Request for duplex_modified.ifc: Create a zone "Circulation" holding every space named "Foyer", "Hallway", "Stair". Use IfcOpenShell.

First a look at what the model holds.

```python
import ifcopenshell

model = ifcopenshell.open("duplex_modified.ifc")
print(model.schema)
seen = {}
for space in model.by_type("IfcSpace"):
    seen[space.LongName] = seen.get(space.LongName, 0) + 1
for name, count in sorted(seen.items(), key=str):
    print(count, "x", name)
print("zones:", [z.Name for z in model.by_type("IfcZone")][:20])
```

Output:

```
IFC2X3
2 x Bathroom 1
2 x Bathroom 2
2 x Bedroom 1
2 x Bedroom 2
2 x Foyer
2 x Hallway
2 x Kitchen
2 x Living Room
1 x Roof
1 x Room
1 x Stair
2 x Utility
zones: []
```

```python
import ifcopenshell
import ifcopenshell.api.group
import ifcopenshell.api.root

model = ifcopenshell.open("duplex_modified.ifc")

names = {"Foyer", "Hallway", "Stair"}
spaces = [s for s in model.by_type("IfcSpace") if s.LongName in names]

zone = ifcopenshell.api.root.create_entity(model, ifc_class="IfcZone", name="Circulation")
ifcopenshell.api.group.assign_group(model, products=spaces, group=zone)
print(len(spaces), "spaces in", zone.Name)

model.write("duplex_modified_updated.ifc")
```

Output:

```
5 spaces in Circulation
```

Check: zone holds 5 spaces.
